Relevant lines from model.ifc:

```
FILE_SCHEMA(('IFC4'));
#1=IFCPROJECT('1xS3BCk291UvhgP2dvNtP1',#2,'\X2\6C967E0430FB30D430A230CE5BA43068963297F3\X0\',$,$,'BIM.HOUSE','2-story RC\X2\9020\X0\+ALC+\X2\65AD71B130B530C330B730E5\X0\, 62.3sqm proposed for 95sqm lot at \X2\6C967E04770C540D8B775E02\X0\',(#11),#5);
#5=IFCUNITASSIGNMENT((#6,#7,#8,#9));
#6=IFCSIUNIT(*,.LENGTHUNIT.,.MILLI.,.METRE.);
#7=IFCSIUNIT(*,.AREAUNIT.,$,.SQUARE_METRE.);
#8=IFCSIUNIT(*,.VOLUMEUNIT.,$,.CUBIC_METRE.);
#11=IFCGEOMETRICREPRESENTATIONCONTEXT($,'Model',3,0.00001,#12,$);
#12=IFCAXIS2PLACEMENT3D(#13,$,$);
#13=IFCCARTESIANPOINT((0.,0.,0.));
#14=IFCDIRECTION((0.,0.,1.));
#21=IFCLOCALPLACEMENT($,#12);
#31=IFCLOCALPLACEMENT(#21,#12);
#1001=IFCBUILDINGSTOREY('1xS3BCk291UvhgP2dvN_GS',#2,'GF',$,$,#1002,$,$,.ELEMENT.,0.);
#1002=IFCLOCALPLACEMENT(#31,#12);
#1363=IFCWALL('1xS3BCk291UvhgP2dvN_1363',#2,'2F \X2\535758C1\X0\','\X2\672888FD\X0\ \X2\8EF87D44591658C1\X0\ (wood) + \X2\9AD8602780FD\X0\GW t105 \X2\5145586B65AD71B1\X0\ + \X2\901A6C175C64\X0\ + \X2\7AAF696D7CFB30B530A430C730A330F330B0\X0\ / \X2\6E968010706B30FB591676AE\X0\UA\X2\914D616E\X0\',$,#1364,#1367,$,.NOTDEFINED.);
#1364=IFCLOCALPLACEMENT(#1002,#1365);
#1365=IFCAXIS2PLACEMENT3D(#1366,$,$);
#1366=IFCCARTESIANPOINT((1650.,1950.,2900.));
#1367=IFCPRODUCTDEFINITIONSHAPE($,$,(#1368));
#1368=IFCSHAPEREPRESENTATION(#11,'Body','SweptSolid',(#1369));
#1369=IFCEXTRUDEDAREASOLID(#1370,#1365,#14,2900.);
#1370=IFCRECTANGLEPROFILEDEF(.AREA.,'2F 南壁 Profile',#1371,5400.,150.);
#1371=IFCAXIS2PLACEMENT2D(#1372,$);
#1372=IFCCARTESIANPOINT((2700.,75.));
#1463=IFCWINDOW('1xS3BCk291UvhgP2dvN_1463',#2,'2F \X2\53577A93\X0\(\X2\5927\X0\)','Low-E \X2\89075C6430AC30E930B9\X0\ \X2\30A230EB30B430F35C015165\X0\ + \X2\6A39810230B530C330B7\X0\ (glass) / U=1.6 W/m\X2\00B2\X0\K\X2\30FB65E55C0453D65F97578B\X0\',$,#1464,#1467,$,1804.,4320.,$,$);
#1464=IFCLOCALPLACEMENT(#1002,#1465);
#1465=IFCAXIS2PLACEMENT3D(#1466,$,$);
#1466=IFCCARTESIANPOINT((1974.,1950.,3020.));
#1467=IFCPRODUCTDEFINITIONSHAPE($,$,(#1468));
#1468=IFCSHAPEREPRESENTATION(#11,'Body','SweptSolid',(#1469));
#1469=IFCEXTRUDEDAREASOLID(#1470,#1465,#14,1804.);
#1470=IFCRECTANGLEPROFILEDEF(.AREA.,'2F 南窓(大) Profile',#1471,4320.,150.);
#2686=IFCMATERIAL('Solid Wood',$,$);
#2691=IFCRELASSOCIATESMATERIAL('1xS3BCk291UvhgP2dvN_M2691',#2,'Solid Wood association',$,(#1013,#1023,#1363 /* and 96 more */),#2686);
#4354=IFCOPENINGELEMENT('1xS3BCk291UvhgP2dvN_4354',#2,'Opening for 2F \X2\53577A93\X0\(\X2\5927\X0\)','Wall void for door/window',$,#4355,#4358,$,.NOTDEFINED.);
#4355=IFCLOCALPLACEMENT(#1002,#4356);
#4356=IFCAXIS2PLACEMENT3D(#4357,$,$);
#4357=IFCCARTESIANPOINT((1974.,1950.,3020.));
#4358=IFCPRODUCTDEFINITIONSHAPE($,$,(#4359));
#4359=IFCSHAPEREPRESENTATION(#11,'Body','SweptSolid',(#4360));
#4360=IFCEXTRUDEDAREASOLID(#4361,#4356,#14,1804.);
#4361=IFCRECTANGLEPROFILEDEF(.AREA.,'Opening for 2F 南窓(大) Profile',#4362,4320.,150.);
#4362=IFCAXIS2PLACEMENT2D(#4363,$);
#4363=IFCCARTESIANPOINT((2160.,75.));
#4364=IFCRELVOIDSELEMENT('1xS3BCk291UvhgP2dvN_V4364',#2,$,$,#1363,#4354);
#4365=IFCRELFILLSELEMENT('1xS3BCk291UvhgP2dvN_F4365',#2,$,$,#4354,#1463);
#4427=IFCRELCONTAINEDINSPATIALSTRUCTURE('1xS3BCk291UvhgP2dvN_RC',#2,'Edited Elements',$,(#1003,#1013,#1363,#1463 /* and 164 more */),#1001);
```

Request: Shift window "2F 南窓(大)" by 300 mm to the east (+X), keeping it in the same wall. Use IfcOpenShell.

```python
import ifcopenshell
import ifcopenshell.api.geometry
import ifcopenshell.util.placement

model = ifcopenshell.open("model.ifc")

window = model.by_guid("1xS3BCk291UvhgP2dvN_1463")
opening = window.FillsVoids[0].RelatingOpeningElement
wall = opening.VoidsElements[0].RelatingBuildingElement

wall_matrix = ifcopenshell.util.placement.get_local_placement(wall.ObjectPlacement)
shift = wall_matrix[:3, 0] * 300.0
before = ifcopenshell.util.placement.get_local_placement(window.ObjectPlacement)[:3, 3].copy()

# The window is not placed relative to its opening, so move both.
for product in (opening, window):
    matrix = ifcopenshell.util.placement.get_local_placement(product.ObjectPlacement)
    matrix[:3, 3] += shift
    ifcopenshell.api.geometry.edit_object_placement(model, product=product, matrix=matrix, is_si=False)

after = ifcopenshell.util.placement.get_local_placement(window.ObjectPlacement)[:3, 3]
print("window moved by", (after - before).round(3) + 0.0)

model.write("model_v2.ifc")
```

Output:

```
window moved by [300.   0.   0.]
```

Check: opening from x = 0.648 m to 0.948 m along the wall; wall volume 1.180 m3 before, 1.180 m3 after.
